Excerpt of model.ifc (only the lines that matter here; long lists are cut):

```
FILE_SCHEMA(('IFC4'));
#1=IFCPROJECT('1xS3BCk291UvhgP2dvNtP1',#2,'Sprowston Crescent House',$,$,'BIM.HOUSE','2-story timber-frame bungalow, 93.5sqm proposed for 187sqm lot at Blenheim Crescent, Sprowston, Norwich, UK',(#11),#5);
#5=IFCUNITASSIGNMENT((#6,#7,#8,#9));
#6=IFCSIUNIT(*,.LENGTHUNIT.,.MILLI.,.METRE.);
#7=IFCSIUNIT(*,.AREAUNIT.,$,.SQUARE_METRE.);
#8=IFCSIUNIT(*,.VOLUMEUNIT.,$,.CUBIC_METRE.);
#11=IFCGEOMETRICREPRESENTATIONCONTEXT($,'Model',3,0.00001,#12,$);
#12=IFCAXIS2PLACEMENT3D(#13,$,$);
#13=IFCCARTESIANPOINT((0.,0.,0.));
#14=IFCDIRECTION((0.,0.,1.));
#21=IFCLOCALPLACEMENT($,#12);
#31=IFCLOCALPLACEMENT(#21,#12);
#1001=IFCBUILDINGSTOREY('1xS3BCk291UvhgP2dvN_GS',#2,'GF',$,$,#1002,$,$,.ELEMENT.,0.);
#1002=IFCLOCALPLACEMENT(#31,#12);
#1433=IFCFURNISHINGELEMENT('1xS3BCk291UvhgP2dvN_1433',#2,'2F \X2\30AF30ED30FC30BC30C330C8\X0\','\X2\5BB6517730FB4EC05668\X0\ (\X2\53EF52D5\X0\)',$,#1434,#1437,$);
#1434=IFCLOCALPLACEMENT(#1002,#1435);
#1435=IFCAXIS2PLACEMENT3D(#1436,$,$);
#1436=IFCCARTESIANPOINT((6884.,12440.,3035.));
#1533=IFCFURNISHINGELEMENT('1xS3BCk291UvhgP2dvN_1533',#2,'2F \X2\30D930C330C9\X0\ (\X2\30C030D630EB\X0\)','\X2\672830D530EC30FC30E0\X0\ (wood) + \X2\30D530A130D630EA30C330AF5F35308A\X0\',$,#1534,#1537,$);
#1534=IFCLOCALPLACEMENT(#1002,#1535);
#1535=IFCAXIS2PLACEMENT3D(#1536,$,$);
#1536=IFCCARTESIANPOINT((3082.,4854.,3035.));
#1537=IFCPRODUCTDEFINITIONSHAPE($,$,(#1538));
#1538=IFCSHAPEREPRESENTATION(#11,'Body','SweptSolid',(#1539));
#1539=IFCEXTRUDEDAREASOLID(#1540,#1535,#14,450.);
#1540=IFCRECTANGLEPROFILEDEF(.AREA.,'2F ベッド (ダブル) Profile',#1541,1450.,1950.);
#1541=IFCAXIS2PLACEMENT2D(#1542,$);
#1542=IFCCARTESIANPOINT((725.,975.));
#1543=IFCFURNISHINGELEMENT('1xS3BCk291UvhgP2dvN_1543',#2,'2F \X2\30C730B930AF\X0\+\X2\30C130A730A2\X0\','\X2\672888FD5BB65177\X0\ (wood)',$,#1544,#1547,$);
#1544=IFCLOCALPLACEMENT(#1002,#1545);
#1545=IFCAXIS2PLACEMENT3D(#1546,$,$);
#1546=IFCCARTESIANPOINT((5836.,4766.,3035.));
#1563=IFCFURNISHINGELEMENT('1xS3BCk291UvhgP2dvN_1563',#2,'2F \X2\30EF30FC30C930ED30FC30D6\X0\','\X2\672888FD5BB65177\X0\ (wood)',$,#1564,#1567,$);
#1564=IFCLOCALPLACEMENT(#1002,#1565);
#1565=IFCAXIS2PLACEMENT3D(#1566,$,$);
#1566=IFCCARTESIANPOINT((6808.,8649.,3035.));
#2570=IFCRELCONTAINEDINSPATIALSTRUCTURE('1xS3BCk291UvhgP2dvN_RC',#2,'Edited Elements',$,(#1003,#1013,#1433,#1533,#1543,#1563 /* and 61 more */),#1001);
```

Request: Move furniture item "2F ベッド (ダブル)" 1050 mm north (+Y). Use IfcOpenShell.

```python
import ifcopenshell
import ifcopenshell.api.geometry
import ifcopenshell.util.placement

model = ifcopenshell.open("model.ifc")

item = model.by_id(1533)
matrix = ifcopenshell.util.placement.get_local_placement(item.ObjectPlacement)
matrix[1, 3] += 1050.0
ifcopenshell.api.geometry.edit_object_placement(model, product=item, matrix=matrix, is_si=False)

print(ifcopenshell.util.placement.get_local_placement(item.ObjectPlacement).round(3) + 0.0)

model.write("model_rev.ifc")
```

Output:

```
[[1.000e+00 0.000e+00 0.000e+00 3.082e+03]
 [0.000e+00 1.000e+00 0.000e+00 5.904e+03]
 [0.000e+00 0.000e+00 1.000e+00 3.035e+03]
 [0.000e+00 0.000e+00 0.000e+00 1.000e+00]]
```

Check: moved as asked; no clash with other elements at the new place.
